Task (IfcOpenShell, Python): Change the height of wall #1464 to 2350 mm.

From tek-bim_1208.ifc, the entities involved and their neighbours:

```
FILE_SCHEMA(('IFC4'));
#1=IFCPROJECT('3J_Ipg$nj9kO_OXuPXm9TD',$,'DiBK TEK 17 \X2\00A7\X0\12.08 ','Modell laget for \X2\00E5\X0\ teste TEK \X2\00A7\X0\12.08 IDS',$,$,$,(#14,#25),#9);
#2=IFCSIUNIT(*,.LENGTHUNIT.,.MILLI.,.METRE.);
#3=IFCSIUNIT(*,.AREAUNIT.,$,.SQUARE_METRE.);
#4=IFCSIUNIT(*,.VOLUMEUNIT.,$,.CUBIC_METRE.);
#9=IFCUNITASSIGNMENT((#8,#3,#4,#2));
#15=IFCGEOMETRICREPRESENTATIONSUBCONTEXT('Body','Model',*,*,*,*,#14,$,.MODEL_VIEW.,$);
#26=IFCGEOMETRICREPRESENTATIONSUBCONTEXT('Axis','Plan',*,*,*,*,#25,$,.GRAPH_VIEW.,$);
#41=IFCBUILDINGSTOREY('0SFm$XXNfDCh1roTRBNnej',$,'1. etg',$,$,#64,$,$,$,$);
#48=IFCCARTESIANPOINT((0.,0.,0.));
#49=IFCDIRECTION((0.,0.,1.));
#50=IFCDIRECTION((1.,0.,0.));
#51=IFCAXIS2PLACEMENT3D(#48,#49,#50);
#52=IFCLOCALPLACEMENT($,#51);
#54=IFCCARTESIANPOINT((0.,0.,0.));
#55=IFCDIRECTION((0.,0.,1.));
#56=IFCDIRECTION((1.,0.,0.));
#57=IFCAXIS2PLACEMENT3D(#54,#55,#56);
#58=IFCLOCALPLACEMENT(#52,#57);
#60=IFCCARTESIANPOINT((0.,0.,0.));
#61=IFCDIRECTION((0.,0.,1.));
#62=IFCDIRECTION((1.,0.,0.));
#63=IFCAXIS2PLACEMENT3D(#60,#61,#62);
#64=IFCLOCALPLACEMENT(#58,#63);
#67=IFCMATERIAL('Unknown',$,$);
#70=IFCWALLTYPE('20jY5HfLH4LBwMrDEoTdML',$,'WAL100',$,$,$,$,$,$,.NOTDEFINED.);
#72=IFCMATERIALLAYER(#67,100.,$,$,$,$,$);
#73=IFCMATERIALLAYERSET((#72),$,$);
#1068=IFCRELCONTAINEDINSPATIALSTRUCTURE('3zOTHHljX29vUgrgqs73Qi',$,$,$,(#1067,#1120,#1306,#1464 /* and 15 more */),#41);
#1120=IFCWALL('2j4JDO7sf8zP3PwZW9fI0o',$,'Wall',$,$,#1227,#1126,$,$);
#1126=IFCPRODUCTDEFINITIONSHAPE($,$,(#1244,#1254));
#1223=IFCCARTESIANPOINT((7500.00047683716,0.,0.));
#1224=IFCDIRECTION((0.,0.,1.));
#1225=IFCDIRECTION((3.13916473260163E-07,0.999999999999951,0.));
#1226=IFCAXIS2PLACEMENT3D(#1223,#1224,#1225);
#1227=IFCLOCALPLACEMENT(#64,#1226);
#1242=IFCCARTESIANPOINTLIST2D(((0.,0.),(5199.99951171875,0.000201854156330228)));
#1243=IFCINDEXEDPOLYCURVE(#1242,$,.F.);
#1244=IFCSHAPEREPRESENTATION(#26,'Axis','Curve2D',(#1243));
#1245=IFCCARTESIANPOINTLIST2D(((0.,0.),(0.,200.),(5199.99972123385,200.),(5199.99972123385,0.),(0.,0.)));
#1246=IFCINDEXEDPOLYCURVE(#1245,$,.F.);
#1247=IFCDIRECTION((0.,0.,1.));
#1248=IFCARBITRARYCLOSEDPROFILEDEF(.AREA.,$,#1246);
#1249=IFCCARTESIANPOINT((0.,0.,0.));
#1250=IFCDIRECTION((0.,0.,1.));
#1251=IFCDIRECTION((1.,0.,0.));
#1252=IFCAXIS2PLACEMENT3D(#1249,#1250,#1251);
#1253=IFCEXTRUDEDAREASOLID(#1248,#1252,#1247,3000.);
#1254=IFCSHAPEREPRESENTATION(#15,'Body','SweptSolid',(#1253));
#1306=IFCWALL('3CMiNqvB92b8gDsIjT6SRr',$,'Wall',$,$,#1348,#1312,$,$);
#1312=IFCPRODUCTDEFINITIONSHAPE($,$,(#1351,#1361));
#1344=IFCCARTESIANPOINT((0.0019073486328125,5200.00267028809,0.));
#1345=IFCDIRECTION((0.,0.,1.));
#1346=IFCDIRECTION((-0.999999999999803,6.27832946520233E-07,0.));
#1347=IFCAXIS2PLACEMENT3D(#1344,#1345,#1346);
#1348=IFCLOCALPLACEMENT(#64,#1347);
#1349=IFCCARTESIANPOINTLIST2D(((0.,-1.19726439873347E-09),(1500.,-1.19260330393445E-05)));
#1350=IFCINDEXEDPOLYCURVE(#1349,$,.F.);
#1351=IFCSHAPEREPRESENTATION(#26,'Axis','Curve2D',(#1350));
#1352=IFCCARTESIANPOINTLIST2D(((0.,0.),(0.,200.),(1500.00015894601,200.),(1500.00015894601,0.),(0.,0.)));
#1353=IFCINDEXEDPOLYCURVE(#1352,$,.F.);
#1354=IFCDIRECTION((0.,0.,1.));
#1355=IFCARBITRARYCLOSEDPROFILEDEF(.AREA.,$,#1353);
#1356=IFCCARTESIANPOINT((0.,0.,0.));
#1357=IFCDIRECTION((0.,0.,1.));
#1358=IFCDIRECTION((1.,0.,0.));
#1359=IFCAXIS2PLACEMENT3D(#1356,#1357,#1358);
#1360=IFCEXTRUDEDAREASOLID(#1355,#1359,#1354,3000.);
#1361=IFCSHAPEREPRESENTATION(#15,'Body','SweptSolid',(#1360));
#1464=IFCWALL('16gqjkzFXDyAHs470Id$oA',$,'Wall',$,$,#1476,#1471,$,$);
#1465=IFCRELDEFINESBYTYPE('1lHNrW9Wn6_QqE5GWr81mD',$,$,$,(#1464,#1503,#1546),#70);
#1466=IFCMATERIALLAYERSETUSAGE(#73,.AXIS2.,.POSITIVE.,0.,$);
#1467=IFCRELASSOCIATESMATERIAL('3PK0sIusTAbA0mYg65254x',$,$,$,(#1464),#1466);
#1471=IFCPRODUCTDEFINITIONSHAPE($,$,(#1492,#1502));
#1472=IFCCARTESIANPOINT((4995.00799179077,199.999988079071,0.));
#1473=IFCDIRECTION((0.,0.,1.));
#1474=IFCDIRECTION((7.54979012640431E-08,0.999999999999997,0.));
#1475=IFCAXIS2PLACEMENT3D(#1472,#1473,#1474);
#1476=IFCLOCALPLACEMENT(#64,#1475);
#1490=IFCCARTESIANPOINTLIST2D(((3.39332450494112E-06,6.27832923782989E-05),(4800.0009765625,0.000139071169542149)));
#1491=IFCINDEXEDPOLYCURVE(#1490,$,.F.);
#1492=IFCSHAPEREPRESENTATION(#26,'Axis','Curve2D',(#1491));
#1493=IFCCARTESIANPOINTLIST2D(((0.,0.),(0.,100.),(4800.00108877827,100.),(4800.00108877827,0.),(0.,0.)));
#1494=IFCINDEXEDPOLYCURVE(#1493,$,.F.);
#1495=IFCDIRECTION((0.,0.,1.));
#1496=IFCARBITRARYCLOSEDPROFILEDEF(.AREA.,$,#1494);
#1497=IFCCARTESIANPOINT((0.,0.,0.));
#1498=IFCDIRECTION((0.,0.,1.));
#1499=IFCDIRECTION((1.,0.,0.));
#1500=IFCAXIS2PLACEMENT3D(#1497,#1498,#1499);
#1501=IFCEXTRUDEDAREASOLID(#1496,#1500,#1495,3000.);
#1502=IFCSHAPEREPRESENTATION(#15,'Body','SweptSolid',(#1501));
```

```python
import ifcopenshell
import ifcopenshell.geom
import ifcopenshell.util.representation
import ifcopenshell.util.shape
import ifcopenshell.util.unit

model = ifcopenshell.open("tek-bim_1208.ifc")
unit_scale = ifcopenshell.util.unit.calculate_unit_scale(model)
settings = ifcopenshell.geom.settings()


def volume(element):
    """Net volume in cubic metres, openings subtracted."""
    shape = ifcopenshell.geom.create_shape(settings, element)
    return ifcopenshell.util.shape.get_volume(shape.geometry)


wall = model.by_guid("16gqjkzFXDyAHs470Id$oA")
before = volume(wall)

body = ifcopenshell.util.representation.get_representation(wall, "Model", "Body")
solid = body.Items[0]
old_height = solid.Depth
solid.Depth = 2.35 / unit_scale
after = volume(wall)

print(f"height {old_height:g} -> {solid.Depth:g}, volume {before:.3f} -> {after:.3f} m3")

model.write("tek-bim_1208_updated.ifc")
```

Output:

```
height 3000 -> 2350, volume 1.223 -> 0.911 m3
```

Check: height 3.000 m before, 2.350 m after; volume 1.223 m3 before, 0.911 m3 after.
